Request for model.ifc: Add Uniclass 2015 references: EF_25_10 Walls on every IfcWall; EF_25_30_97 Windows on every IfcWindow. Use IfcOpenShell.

First a look at what the model holds.

```python
import ifcopenshell

model = ifcopenshell.open("model.ifc")
print(model.schema)
print("classifications:", [c.Name for c in model.by_type("IfcClassification")])
for ifc_class in ("IfcDoor", "IfcRoof", "IfcStair", "IfcWall", "IfcWindow"):
    print(ifc_class, len(model.by_type(ifc_class)))
```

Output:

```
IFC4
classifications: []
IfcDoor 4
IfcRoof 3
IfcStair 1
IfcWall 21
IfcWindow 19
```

```python
import ifcopenshell
import ifcopenshell.api.classification

model = ifcopenshell.open("model.ifc")

system = ifcopenshell.api.classification.add_classification(model, classification="Uniclass 2015")

codes = {
    "IfcWall": ("EF_25_10", "Walls"),
    "IfcWindow": ("EF_25_30_97", "Windows"),
}
for ifc_class, (code, name) in codes.items():
    products = model.by_type(ifc_class)
    ifcopenshell.api.classification.add_reference(
        model, products=products, classification=system, identification=code, name=name
    )
    print(code, len(products))

model.write("model_updated.ifc")
```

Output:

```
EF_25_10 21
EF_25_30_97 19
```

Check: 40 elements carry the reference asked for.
